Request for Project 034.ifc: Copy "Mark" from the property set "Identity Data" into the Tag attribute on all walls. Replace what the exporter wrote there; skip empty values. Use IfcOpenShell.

First a look at what the model holds.

```python
import ifcopenshell
import ifcopenshell.util.element

model = ifcopenshell.open("Project 034.ifc")
print(model.schema)
walls = model.by_type("IfcWall")
print(len(walls), "walls")
for e in walls[:8]:
    source = ifcopenshell.util.element.get_pset(e, "Identity Data", "Mark")
    target = e.Tag
    print(e.id(), repr(source), repr(target), sep=" | ")
```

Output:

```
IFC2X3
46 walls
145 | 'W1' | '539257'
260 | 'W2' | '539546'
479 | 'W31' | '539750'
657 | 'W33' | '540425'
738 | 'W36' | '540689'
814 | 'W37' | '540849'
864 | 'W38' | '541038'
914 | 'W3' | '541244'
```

```python
import ifcopenshell
import ifcopenshell.util.element

model = ifcopenshell.open("Project 034.ifc")

count = 0
for e in model.by_type("IfcWall"):
    value = ifcopenshell.util.element.get_pset(e, "Identity Data", "Mark")
    current = e.Tag
    if not value or not value.strip() or current == value:
        continue
    e.Tag = value
    count += 1

print(count, "walls updated")

model.write("Project 034_rev.ifc")
```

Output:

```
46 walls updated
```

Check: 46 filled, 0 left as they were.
